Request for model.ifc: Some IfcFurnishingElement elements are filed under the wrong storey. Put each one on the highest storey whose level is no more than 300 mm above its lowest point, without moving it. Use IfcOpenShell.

First a look at what the model holds.

```python
import ifcopenshell
import ifcopenshell.util.element
import ifcopenshell.util.placement

model = ifcopenshell.open("model.ifc")
print(model.schema)
for storey in model.by_type("IfcBuildingStorey"):
    level = ifcopenshell.util.placement.get_storey_elevation(storey)
    count = sum(e.is_a("IfcFurnishingElement") for e in ifcopenshell.util.element.get_contained(storey))
    print(storey.id(), storey.Name, round(level, 3), count, sep=" | ")
```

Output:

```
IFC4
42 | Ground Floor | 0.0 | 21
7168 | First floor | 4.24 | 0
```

```python
import ifcopenshell
import ifcopenshell.api.spatial
import ifcopenshell.geom
import ifcopenshell.util.element
import ifcopenshell.util.placement
import ifcopenshell.util.shape
import ifcopenshell.util.unit

model = ifcopenshell.open("model.ifc")
unit_scale = ifcopenshell.util.unit.calculate_unit_scale(model)
settings = ifcopenshell.geom.settings()

levels = sorted(
    ((ifcopenshell.util.placement.get_storey_elevation(s) * unit_scale, s) for s in model.by_type("IfcBuildingStorey")),
    key=lambda pair: pair[0],
)

for e in model.by_type("IfcFurnishingElement"):
    current = e.ContainedInStructure[0].RelatingStructure if e.ContainedInStructure else None
    if current is None or not current.is_a("IfcBuildingStorey"):
        continue
    shape = ifcopenshell.geom.create_shape(settings, e)
    bottom = ifcopenshell.util.shape.get_shape_bottom_elevation(shape, shape.geometry)
    below = [s for level, s in levels if level <= bottom + 0.3]
    storey = below[-1] if below else levels[0][1]
    if storey != current:
        # assign_container keeps the world position.
        ifcopenshell.api.spatial.assign_container(model, products=[e], relating_structure=storey)
        print(e.id(), current.Name, "->", storey.Name)

model.write("model_rev.ifc")
```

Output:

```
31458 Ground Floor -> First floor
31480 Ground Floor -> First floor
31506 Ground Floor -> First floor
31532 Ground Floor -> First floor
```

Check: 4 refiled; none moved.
